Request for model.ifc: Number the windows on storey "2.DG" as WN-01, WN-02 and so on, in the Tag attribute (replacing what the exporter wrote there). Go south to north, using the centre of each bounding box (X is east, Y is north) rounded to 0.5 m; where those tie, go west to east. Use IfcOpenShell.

First a look at what the model holds.

```python
import ifcopenshell
import ifcopenshell.util.element
import ifcopenshell.util.placement

model = ifcopenshell.open("model.ifc")
print(model.schema)
storey = next(s for s in model.by_type("IfcBuildingStorey") if s.Name == "2.DG")
windows = [e for e in ifcopenshell.util.element.get_decomposition(storey) if e.is_a("IfcWindow")]
for e in sorted(windows, key=lambda e: e.id()):
    origin = ifcopenshell.util.placement.get_local_placement(e.ObjectPlacement)[:3, 3]
    print(e.id(), e.Tag, e.Name, origin.round(2) + 0.0, sep=" | ")
```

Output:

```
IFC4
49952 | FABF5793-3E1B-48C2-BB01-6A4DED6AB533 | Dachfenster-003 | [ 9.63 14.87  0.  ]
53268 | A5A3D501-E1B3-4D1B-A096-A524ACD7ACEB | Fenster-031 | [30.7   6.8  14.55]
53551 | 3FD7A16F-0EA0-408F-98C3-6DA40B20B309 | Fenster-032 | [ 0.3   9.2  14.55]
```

```python
import ifcopenshell
import ifcopenshell.geom
import ifcopenshell.util.element
import ifcopenshell.util.shape

model = ifcopenshell.open("model.ifc")
settings = ifcopenshell.geom.settings()
settings.set("use-world-coords", True)


def centre(element):
    shape = ifcopenshell.geom.create_shape(settings, element)
    return ifcopenshell.util.shape.get_bbox_centroid(shape.geometry)


storey = next(s for s in model.by_type("IfcBuildingStorey") if s.Name == "2.DG")
windows = [e for e in ifcopenshell.util.element.get_decomposition(storey) if e.is_a("IfcWindow")]

# Insertion points can sit at a corner or the storey origin, so sort by the geometry (in metres).
centres = {e: centre(e) for e in windows}
windows.sort(key=lambda e: (round(centres[e][1] / 0.5), centres[e][0]))

for i, e in enumerate(windows, start=1):
    number = f"WN-{i:02d}"
    e.Tag = number
    print(e.id(), number)

model.write("model_v2.ifc")
```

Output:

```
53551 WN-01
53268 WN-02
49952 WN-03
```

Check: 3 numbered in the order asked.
